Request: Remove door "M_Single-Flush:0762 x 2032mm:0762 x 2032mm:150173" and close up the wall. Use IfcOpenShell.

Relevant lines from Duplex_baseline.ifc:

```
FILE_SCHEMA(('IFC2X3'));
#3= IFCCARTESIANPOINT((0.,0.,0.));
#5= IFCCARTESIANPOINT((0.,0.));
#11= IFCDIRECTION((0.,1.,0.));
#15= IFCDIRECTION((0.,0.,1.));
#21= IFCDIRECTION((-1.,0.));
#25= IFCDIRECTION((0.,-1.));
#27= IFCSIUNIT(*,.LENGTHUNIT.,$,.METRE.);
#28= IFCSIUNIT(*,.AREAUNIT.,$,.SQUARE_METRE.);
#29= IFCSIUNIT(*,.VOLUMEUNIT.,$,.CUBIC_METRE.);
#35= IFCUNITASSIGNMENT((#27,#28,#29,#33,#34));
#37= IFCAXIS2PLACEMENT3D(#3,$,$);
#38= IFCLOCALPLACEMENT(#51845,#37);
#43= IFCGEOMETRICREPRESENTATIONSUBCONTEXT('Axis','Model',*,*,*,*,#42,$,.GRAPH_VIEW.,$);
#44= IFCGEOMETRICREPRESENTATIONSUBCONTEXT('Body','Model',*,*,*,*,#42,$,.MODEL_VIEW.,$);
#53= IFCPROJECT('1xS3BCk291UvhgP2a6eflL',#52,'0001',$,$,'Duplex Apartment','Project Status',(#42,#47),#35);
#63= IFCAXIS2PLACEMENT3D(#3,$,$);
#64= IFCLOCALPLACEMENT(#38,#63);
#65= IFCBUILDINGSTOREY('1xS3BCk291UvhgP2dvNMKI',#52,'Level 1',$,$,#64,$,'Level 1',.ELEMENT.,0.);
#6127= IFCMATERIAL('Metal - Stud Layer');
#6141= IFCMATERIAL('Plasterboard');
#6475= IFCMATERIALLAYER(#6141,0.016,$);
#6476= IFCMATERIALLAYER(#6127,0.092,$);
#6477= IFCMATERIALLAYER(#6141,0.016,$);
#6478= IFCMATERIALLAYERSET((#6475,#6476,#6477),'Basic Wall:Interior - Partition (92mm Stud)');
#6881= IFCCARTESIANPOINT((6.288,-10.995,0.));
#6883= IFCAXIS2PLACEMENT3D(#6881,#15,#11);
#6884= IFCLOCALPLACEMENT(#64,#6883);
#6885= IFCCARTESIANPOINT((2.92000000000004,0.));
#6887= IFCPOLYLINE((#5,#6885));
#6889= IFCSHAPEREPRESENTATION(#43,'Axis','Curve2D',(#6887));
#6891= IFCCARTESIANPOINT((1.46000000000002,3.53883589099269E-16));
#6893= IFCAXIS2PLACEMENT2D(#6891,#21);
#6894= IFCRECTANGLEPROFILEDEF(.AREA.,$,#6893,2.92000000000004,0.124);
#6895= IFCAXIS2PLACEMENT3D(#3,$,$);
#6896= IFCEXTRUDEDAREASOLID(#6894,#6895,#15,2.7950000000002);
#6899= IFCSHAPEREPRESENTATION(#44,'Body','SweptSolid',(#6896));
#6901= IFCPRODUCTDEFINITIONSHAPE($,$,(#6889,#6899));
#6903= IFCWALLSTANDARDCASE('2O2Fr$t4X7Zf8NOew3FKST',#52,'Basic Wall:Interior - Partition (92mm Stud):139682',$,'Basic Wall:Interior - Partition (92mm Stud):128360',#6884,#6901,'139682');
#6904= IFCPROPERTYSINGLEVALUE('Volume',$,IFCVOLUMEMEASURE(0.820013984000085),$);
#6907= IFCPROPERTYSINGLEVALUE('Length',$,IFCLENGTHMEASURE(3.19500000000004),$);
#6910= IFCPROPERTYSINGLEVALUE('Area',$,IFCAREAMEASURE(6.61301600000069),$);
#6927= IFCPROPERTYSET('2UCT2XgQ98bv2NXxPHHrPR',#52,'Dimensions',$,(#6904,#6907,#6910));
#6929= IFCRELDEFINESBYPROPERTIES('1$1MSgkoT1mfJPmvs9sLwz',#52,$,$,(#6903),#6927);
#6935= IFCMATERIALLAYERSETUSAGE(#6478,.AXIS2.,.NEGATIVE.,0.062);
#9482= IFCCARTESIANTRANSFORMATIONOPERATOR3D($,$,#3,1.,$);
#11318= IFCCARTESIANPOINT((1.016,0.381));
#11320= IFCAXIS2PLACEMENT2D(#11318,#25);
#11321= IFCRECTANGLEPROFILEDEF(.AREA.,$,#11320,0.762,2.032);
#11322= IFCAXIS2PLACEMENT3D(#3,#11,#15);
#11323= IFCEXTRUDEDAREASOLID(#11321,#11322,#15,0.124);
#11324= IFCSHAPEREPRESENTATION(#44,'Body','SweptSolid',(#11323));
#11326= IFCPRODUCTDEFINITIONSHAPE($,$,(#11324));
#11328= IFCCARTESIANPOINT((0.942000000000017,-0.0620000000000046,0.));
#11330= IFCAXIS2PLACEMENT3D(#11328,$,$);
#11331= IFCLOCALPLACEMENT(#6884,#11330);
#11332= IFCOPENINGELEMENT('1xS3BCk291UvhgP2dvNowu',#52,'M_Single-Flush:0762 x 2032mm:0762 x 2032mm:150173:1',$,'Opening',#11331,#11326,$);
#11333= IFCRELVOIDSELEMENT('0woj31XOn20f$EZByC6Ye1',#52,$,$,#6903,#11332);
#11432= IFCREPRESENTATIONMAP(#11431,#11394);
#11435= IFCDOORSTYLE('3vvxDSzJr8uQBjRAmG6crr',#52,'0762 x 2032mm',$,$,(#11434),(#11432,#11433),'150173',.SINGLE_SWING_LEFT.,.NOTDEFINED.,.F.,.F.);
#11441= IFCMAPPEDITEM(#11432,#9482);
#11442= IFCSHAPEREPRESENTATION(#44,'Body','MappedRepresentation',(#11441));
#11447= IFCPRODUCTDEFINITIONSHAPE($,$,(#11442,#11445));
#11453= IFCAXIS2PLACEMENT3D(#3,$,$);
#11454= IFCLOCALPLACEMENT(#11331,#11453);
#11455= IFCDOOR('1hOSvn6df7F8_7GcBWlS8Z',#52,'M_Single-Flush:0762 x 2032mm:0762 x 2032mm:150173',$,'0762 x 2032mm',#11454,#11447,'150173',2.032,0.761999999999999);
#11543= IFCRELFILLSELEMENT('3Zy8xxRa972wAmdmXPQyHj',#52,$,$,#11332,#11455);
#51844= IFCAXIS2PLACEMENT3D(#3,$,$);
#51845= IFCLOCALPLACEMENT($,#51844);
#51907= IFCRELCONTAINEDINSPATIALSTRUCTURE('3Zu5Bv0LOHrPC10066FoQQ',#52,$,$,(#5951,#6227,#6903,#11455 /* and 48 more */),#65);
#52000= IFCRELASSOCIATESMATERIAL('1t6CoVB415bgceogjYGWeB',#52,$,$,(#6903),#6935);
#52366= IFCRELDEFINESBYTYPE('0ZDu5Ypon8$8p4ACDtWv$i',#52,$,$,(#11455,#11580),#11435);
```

```python
import ifcopenshell
import ifcopenshell.api.feature
import ifcopenshell.api.pset
import ifcopenshell.api.root
import ifcopenshell.geom
import ifcopenshell.util.element
import ifcopenshell.util.shape
import ifcopenshell.util.unit

model = ifcopenshell.open("Duplex_baseline.ifc")
area_scale = ifcopenshell.util.unit.calculate_unit_scale(model, "AREAUNIT")
volume_scale = ifcopenshell.util.unit.calculate_unit_scale(model, "VOLUMEUNIT")
settings = ifcopenshell.geom.settings()


def volume(element):
    """Net volume in cubic metres, openings subtracted."""
    shape = ifcopenshell.geom.create_shape(settings, element)
    return ifcopenshell.util.shape.get_volume(shape.geometry)


door = model.by_guid("1hOSvn6df7F8_7GcBWlS8Z")
opening = door.FillsVoids[0].RelatingOpeningElement
wall = opening.VoidsElements[0].RelatingBuildingElement
before = volume(wall)

ifcopenshell.api.root.remove_product(model, product=door)
ifcopenshell.api.feature.remove_feature(model, feature=opening)

after = volume(wall)
thickness = 0.124  # wall thickness in metres

# Update the wall's stored quantities.
pset = model.by_id(ifcopenshell.util.element.get_pset(wall, "Dimensions", should_inherit=False)["id"])
ifcopenshell.api.pset.edit_pset(model, pset=pset, properties={
    "Volume": model.create_entity("IfcVolumeMeasure", after / volume_scale),
    "Area": model.create_entity("IfcAreaMeasure", after / thickness / area_scale),
})

print(f"wall volume {before:.3f} -> {after:.3f} m3")

model.write("Duplex_baseline_rev.ifc")
```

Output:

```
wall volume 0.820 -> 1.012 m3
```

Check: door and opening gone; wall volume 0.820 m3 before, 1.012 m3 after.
